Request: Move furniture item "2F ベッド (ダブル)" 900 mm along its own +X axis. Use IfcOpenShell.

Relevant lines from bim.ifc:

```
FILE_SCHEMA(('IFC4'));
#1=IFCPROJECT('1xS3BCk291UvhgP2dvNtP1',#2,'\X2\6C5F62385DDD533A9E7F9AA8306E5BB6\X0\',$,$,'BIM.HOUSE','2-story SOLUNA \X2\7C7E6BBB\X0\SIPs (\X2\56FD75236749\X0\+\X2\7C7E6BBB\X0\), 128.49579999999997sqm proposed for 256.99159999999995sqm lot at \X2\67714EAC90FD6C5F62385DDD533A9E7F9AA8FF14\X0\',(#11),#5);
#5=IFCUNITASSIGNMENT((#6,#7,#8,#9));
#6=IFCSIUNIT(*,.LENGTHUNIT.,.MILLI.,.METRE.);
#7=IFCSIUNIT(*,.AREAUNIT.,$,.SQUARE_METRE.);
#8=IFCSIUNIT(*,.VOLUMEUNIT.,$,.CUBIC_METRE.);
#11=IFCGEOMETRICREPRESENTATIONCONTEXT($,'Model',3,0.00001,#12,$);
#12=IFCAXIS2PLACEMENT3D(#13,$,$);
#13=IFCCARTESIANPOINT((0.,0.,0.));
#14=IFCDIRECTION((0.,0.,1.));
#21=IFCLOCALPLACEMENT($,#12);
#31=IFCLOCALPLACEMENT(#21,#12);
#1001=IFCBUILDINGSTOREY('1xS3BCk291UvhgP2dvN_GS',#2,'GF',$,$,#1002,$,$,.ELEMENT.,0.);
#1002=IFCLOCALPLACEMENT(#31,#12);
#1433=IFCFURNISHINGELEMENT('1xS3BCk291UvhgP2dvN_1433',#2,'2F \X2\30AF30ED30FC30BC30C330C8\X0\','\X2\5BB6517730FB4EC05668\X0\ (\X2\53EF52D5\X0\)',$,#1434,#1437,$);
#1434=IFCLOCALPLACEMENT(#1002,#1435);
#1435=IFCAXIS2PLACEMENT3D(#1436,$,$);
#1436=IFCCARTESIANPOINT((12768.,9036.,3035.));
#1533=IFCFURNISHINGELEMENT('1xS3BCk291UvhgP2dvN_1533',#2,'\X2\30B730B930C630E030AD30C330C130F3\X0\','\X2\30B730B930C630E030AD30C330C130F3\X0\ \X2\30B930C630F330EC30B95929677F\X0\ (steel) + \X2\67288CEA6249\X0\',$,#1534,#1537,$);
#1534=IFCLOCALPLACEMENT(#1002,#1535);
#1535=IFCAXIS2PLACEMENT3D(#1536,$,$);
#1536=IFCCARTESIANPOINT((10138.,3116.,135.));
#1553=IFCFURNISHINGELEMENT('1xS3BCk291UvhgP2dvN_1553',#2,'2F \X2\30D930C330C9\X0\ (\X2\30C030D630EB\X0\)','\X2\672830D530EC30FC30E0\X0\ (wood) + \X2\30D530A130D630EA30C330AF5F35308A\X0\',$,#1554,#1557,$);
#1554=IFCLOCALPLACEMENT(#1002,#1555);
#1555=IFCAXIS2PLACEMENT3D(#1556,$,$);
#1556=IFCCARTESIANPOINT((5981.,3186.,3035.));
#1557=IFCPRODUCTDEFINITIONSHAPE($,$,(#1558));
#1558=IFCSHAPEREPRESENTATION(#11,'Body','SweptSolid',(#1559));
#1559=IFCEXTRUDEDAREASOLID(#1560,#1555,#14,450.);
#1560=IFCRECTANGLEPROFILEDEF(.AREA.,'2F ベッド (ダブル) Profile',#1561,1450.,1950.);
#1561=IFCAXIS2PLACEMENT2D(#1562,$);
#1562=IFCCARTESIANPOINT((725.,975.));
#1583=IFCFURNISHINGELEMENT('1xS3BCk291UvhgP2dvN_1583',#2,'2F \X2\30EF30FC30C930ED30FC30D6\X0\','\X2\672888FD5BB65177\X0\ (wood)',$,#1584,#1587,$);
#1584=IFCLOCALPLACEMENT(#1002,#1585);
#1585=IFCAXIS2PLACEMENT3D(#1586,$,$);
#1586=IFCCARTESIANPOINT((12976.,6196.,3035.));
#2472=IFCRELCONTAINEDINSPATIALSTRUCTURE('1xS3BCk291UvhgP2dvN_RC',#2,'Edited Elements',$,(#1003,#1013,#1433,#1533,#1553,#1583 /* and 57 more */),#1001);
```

```python
import ifcopenshell
import ifcopenshell.api.geometry
import ifcopenshell.util.placement
import ifcopenshell.util.unit

model = ifcopenshell.open("bim.ifc")
unit_scale = ifcopenshell.util.unit.calculate_unit_scale(model)

item = model.by_guid("1xS3BCk291UvhgP2dvN_1553")
matrix = ifcopenshell.util.placement.get_local_placement(item.ObjectPlacement)
matrix[:3, 3] += matrix[:3, 0] * 0.9 / unit_scale
ifcopenshell.api.geometry.edit_object_placement(model, product=item, matrix=matrix, is_si=False)

print(ifcopenshell.util.placement.get_local_placement(item.ObjectPlacement).round(3) + 0.0)

model.write("bim_rev.ifc")
```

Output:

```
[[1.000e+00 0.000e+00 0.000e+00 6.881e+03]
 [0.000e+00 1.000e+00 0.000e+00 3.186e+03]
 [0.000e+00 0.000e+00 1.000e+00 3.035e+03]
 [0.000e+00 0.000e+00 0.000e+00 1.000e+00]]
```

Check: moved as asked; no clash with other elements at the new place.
